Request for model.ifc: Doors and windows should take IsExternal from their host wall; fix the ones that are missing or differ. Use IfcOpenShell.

First a look at what the model holds.

```python
import ifcopenshell
import ifcopenshell.util.element

model = ifcopenshell.open("model.ifc")
print(model.schema)
seen = {}
for e in model.by_type("IfcDoor") + model.by_type("IfcWindow"):
    if not e.FillsVoids:
        continue
    host = e.FillsVoids[0].RelatingOpeningElement.VoidsElements[0].RelatingBuildingElement
    own = ifcopenshell.util.element.get_pset(e, f"Pset_{e.is_a()[3:].removesuffix('StandardCase')}Common", "IsExternal")
    wall = ifcopenshell.util.element.get_pset(host, "Pset_WallCommon", "IsExternal")
    seen[e.is_a(), own, wall] = seen.get((e.is_a(), own, wall), 0) + 1
for (cls, own, wall), count in sorted(seen.items(), key=str):
    print(count, cls, "IsExternal:", own, "| host wall:", wall)
```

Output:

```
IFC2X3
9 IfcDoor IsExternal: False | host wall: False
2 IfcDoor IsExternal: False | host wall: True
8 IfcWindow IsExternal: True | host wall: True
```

```python
import ifcopenshell
import ifcopenshell.api.pset
import ifcopenshell.util.element

model = ifcopenshell.open("model.ifc")

count = 0
for ifc_class, pset_name in (("IfcDoor", "Pset_DoorCommon"), ("IfcWindow", "Pset_WindowCommon")):
    for e in model.by_type(ifc_class):
        if not e.FillsVoids:
            continue
        host = e.FillsVoids[0].RelatingOpeningElement.VoidsElements[0].RelatingBuildingElement
        external = ifcopenshell.util.element.get_pset(host, "Pset_WallCommon", "IsExternal")
        if external is None or ifcopenshell.util.element.get_pset(e, pset_name, "IsExternal") == external:
            continue
        pset = ifcopenshell.api.pset.add_pset(model, product=e, name=pset_name)
        ifcopenshell.api.pset.edit_pset(model, pset=pset, properties={"IsExternal": external})
        count += 1

print(count, "updated")

model.write("model_edited.ifc")
```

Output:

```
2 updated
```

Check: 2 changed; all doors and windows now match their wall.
